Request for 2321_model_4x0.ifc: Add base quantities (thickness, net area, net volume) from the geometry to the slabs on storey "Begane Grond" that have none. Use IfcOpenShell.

First a look at what the model holds.

```python
import ifcopenshell
import ifcopenshell.util.element
import ifcopenshell.util.unit

model = ifcopenshell.open("2321_model_4x0.ifc")
print(model.schema)
for unit_type in ("LENGTHUNIT", "AREAUNIT", "VOLUMEUNIT"):
    print(unit_type, ifcopenshell.util.unit.calculate_unit_scale(model, unit_type))
storey = next(s for s in model.by_type("IfcBuildingStorey") if s.Name == "Begane Grond")
slabs = [e for e in ifcopenshell.util.element.get_decomposition(storey) if e.is_a("IfcSlab")]
for e in sorted(slabs, key=lambda e: e.id()):
    print(e.id(), e.is_a(), e.Name, list(ifcopenshell.util.element.get_psets(e, qtos_only=True)), sep=" | ")
```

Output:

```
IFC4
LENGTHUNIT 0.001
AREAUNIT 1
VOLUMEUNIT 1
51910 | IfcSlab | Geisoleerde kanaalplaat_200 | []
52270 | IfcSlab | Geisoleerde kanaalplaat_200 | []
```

```python
import ifcopenshell
import ifcopenshell.api.pset
import ifcopenshell.geom
import ifcopenshell.util.element
import ifcopenshell.util.shape
import ifcopenshell.util.unit

model = ifcopenshell.open("2321_model_4x0.ifc")
unit_scale = ifcopenshell.util.unit.calculate_unit_scale(model)
area_scale = ifcopenshell.util.unit.calculate_unit_scale(model, "AREAUNIT")
volume_scale = ifcopenshell.util.unit.calculate_unit_scale(model, "VOLUMEUNIT")
settings = ifcopenshell.geom.settings()

storey = next(s for s in model.by_type("IfcBuildingStorey") if s.Name == "Begane Grond")
slabs = [e for e in ifcopenshell.util.element.get_decomposition(storey) if e.is_a("IfcSlab")]

for e in sorted(slabs, key=lambda e: e.id()):
    if ifcopenshell.util.element.get_psets(e, qtos_only=True, should_inherit=False):
        continue
    # Geometry comes back in metres, in the element's own axes.
    shape = ifcopenshell.geom.create_shape(settings, e)
    values = {
        "Width": ifcopenshell.util.shape.get_z(shape.geometry) / unit_scale,
        "NetArea": ifcopenshell.util.shape.get_footprint_area(shape.geometry) / area_scale,
        "NetVolume": ifcopenshell.util.shape.get_volume(shape.geometry) / volume_scale,
    }
    qto = ifcopenshell.api.pset.add_qto(model, product=e, name="Qto_SlabBaseQuantities")
    ifcopenshell.api.pset.edit_qto(model, qto=qto, properties=values)
    print(e.id(), {k: round(v, 3) for k, v in values.items()})

model.write("2321_model_4x0_rev.ifc")
```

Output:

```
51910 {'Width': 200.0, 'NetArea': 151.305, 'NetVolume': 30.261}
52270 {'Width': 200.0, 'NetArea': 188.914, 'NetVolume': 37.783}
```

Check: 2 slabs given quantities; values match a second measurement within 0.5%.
